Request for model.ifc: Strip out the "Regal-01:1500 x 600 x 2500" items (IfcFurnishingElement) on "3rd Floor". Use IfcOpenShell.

First a look at what the model holds.

```python
import ifcopenshell
import ifcopenshell.util.element

model = ifcopenshell.open("model.ifc")
print(model.schema)
storey = next(s for s in model.by_type("IfcBuildingStorey") if s.Name == "3rd Floor")
furniture = [e for e in ifcopenshell.util.element.get_decomposition(storey) if e.is_a("IfcFurnishingElement")]
seen = {}
for e in furniture:
    element_type = ifcopenshell.util.element.get_type(e)
    name = element_type.Name if element_type not in (None, e) else None
    seen[name] = seen.get(name, 0) + 1
for name, count in sorted(seen.items(), key=str):
    print(count, "x", name)
```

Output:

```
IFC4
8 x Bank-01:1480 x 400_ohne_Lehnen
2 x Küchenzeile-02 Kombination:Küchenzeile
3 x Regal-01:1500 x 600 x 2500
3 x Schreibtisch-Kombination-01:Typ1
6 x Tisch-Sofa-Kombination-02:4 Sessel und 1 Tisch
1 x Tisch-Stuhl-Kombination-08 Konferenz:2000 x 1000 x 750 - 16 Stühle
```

```python
import ifcopenshell
import ifcopenshell.api.root
import ifcopenshell.util.element

model = ifcopenshell.open("model.ifc")

storey = next(s for s in model.by_type("IfcBuildingStorey") if s.Name == "3rd Floor")
furniture = [e for e in ifcopenshell.util.element.get_decomposition(storey) if e.is_a("IfcFurnishingElement")]
targets = [e for e in furniture if (t := ifcopenshell.util.element.get_type(e)) not in (None, e) and t.Name == "Regal-01:1500 x 600 x 2500"]

for e in targets:
    ifcopenshell.api.root.remove_product(model, product=e)
print(len(targets), "removed")

model.write("model_updated.ifc")
```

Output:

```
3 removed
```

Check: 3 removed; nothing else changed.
